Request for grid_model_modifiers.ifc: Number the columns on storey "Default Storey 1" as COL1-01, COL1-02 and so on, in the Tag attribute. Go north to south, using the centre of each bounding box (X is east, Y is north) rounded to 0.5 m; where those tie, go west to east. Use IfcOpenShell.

First a look at what the model holds.

```python
import ifcopenshell
import ifcopenshell.util.element
import ifcopenshell.util.placement

model = ifcopenshell.open("grid_model_modifiers.ifc")
print(model.schema)
storey = next(s for s in model.by_type("IfcBuildingStorey") if s.Name == "Default Storey 1")
columns = [e for e in ifcopenshell.util.element.get_decomposition(storey) if e.is_a("IfcColumn")]
for e in sorted(columns, key=lambda e: e.id()):
    origin = ifcopenshell.util.placement.get_local_placement(e.ObjectPlacement)[:3, 3]
    print(e.id(), e.Tag, e.Name, origin.round(2) + 0.0, sep=" | ")
```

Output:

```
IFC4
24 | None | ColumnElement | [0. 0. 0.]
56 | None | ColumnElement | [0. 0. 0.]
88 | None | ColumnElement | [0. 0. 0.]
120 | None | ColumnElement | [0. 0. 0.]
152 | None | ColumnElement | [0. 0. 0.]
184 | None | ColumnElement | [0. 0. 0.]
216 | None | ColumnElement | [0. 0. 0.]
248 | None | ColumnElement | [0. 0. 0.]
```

```python
import ifcopenshell
import ifcopenshell.geom
import ifcopenshell.util.element
import ifcopenshell.util.shape

model = ifcopenshell.open("grid_model_modifiers.ifc")
settings = ifcopenshell.geom.settings()
settings.set("use-world-coords", True)


def centre(element):
    shape = ifcopenshell.geom.create_shape(settings, element)
    return ifcopenshell.util.shape.get_bbox_centroid(shape.geometry)


storey = next(s for s in model.by_type("IfcBuildingStorey") if s.Name == "Default Storey 1")
columns = [e for e in ifcopenshell.util.element.get_decomposition(storey) if e.is_a("IfcColumn")]

# Insertion points can sit at a corner or the storey origin, so sort by the geometry (in metres).
centres = {e: centre(e) for e in columns}
columns.sort(key=lambda e: (-round(centres[e][1] / 0.5), centres[e][0]))

for i, e in enumerate(columns, start=1):
    number = f"COL1-{i:02d}"
    e.Tag = number
    print(e.id(), number)

model.write("grid_model_modifiers-out.ifc")
```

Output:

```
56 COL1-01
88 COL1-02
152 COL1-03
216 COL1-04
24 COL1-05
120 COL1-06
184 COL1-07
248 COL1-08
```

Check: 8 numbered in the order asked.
